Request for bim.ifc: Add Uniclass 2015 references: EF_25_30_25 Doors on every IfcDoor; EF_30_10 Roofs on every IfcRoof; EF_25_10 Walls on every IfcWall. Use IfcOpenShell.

First a look at what the model holds.

```python
import ifcopenshell

model = ifcopenshell.open("bim.ifc")
print(model.schema)
print("classifications:", [c.Name for c in model.by_type("IfcClassification")])
for ifc_class in ("IfcDoor", "IfcRoof", "IfcStair", "IfcWall", "IfcWindow"):
    print(ifc_class, len(model.by_type(ifc_class)))
```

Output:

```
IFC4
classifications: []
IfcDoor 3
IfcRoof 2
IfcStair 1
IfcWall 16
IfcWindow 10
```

```python
import ifcopenshell
import ifcopenshell.api.classification

model = ifcopenshell.open("bim.ifc")

system = ifcopenshell.api.classification.add_classification(model, classification="Uniclass 2015")

codes = {
    "IfcDoor": ("EF_25_30_25", "Doors"),
    "IfcRoof": ("EF_30_10", "Roofs"),
    "IfcWall": ("EF_25_10", "Walls"),
}
for ifc_class, (code, name) in codes.items():
    products = model.by_type(ifc_class)
    ifcopenshell.api.classification.add_reference(
        model, products=products, classification=system, identification=code, name=name
    )
    print(code, len(products))

model.write("bim_v2.ifc")
```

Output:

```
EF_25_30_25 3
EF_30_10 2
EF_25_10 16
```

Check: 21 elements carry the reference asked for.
